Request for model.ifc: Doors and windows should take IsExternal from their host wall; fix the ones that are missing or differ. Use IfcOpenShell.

First a look at what the model holds.

```python
import ifcopenshell
import ifcopenshell.util.element

model = ifcopenshell.open("model.ifc")
print(model.schema)
seen = {}
for e in model.by_type("IfcDoor") + model.by_type("IfcWindow"):
    if not e.FillsVoids:
        continue
    host = e.FillsVoids[0].RelatingOpeningElement.VoidsElements[0].RelatingBuildingElement
    own = ifcopenshell.util.element.get_pset(e, f"Pset_{e.is_a()[3:].removesuffix('StandardCase')}Common", "IsExternal")
    wall = ifcopenshell.util.element.get_pset(host, "Pset_WallCommon", "IsExternal")
    seen[e.is_a(), own, wall] = seen.get((e.is_a(), own, wall), 0) + 1
for (cls, own, wall), count in sorted(seen.items(), key=str):
    print(count, cls, "IsExternal:", own, "| host wall:", wall)
```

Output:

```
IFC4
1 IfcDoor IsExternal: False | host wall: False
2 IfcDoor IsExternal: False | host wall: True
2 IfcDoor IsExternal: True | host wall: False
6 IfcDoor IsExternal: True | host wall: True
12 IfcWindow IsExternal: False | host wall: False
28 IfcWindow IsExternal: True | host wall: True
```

```python
import ifcopenshell
import ifcopenshell.api.pset
import ifcopenshell.util.element

model = ifcopenshell.open("model.ifc")

count = 0
for ifc_class, pset_name in (("IfcDoor", "Pset_DoorCommon"), ("IfcWindow", "Pset_WindowCommon")):
    for e in model.by_type(ifc_class):
        if not e.FillsVoids:
            continue
        host = e.FillsVoids[0].RelatingOpeningElement.VoidsElements[0].RelatingBuildingElement
        external = ifcopenshell.util.element.get_pset(host, "Pset_WallCommon", "IsExternal")
        if external is None or ifcopenshell.util.element.get_pset(e, pset_name, "IsExternal") == external:
            continue
        pset = ifcopenshell.api.pset.add_pset(model, product=e, name=pset_name)
        ifcopenshell.api.pset.edit_pset(model, pset=pset, properties={"IsExternal": external})
        count += 1

print(count, "updated")

model.write("model_edited.ifc")
```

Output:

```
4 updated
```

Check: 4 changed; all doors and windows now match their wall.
